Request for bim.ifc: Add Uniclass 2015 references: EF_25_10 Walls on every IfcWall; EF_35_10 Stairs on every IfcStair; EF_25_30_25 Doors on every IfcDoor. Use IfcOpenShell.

First a look at what the model holds.

```python
import ifcopenshell

model = ifcopenshell.open("bim.ifc")
print(model.schema)
print("classifications:", [c.Name for c in model.by_type("IfcClassification")])
for ifc_class in ("IfcDoor", "IfcRoof", "IfcStair", "IfcWall", "IfcWindow"):
    print(ifc_class, len(model.by_type(ifc_class)))
```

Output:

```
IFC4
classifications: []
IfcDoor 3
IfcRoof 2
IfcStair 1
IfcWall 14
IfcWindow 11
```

```python
import ifcopenshell
import ifcopenshell.api.classification

model = ifcopenshell.open("bim.ifc")

system = ifcopenshell.api.classification.add_classification(model, classification="Uniclass 2015")

codes = {
    "IfcWall": ("EF_25_10", "Walls"),
    "IfcStair": ("EF_35_10", "Stairs"),
    "IfcDoor": ("EF_25_30_25", "Doors"),
}
for ifc_class, (code, name) in codes.items():
    products = model.by_type(ifc_class)
    ifcopenshell.api.classification.add_reference(
        model, products=products, classification=system, identification=code, name=name
    )
    print(code, len(products))

model.write("bim_rev.ifc")
```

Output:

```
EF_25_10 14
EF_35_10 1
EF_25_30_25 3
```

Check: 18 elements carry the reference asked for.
